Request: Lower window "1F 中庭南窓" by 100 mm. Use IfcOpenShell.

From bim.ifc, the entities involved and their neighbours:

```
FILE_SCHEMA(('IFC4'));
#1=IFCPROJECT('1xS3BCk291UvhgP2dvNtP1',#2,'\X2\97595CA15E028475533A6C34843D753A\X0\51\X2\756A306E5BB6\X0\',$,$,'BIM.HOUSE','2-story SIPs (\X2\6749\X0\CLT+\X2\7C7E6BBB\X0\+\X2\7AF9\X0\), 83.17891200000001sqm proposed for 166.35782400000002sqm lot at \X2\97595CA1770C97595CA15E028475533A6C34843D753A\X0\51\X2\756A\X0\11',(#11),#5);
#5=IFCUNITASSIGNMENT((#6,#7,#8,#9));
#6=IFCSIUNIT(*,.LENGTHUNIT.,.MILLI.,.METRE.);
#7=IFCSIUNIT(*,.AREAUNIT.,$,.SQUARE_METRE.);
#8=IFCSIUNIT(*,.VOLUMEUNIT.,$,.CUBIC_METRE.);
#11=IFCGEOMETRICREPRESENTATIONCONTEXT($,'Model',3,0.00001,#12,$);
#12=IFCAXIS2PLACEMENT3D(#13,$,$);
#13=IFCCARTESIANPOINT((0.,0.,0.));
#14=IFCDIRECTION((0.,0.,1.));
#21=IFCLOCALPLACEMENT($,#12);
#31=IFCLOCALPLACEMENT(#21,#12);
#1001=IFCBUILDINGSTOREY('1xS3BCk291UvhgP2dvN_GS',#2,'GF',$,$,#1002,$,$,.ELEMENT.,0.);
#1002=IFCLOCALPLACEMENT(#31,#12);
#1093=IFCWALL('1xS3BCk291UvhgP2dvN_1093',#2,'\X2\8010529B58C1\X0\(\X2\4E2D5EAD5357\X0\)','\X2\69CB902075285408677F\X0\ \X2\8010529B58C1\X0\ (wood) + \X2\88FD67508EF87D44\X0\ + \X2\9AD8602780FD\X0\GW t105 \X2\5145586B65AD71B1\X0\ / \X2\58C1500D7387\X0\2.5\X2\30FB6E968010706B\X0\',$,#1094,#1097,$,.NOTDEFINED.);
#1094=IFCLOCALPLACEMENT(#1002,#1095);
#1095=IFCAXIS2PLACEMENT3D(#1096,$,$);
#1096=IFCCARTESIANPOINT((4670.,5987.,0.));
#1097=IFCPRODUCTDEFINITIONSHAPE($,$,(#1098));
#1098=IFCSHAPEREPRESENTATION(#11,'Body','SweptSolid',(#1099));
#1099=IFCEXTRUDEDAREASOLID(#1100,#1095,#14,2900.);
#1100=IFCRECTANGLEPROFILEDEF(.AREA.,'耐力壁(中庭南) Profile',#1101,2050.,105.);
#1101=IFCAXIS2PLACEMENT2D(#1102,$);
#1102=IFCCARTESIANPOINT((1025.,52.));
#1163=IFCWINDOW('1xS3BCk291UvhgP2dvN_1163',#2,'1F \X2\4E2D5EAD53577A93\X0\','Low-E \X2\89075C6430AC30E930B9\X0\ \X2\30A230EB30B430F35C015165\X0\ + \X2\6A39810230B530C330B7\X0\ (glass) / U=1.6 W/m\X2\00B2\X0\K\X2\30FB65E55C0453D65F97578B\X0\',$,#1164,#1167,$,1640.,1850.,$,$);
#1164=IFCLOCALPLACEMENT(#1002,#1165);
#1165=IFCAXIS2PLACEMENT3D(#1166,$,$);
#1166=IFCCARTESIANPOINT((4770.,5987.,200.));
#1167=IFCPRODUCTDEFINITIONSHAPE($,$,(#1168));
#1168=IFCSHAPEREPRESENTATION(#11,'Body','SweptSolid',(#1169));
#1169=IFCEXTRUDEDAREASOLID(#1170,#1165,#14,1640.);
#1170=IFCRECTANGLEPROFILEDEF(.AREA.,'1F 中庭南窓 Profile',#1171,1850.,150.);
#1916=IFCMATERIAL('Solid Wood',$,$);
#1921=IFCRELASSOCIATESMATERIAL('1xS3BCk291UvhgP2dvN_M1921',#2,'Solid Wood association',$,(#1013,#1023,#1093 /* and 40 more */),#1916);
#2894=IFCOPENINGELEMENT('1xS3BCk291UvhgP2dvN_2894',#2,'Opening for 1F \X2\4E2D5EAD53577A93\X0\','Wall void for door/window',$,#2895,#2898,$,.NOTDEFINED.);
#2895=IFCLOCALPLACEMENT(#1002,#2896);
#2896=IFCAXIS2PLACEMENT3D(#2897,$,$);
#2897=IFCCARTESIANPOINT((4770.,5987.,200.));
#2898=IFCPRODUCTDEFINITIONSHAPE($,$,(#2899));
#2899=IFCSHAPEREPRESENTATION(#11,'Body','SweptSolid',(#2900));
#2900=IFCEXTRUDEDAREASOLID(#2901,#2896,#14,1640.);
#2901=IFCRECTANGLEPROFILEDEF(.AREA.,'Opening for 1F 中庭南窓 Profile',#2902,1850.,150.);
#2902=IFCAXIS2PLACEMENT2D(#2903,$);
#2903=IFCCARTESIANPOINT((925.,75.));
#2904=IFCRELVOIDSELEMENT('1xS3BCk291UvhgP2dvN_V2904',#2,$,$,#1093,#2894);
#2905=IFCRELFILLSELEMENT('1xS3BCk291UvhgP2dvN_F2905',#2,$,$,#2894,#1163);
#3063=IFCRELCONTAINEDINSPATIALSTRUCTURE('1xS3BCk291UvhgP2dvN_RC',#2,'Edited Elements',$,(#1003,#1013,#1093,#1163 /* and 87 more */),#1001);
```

```python
import numpy as np
import ifcopenshell
import ifcopenshell.api.geometry
import ifcopenshell.util.placement
import ifcopenshell.util.unit

model = ifcopenshell.open("bim.ifc")
unit_scale = ifcopenshell.util.unit.calculate_unit_scale(model)

window = model.by_guid("1xS3BCk291UvhgP2dvN_1163")
opening = window.FillsVoids[0].RelatingOpeningElement
dz = -0.1 / unit_scale

shift = np.array([0.0, 0.0, dz])
# The window is not placed relative to its opening, so move both.
for product in (opening, window):
    matrix = ifcopenshell.util.placement.get_local_placement(product.ObjectPlacement)
    matrix[:3, 3] += shift
    ifcopenshell.api.geometry.edit_object_placement(model, product=product, matrix=matrix, is_si=False)

print(f"moved by {dz * unit_scale:+.3f} m")

model.write("bim_updated.ifc")
```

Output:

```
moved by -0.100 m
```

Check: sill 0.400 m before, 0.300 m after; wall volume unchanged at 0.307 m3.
